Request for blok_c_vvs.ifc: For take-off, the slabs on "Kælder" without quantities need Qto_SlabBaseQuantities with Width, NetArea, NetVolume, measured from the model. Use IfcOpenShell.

First a look at what the model holds.

```python
import ifcopenshell
import ifcopenshell.util.element
import ifcopenshell.util.unit

model = ifcopenshell.open("blok_c_vvs.ifc")
print(model.schema)
for unit_type in ("LENGTHUNIT", "AREAUNIT", "VOLUMEUNIT"):
    print(unit_type, ifcopenshell.util.unit.calculate_unit_scale(model, unit_type))
storey = next(s for s in model.by_type("IfcBuildingStorey") if s.Name == "Kælder")
slabs = [e for e in ifcopenshell.util.element.get_decomposition(storey) if e.is_a("IfcSlab")]
for e in sorted(slabs, key=lambda e: e.id()):
    print(e.id(), e.is_a(), e.Name, list(ifcopenshell.util.element.get_psets(e, qtos_only=True)), sep=" | ")
```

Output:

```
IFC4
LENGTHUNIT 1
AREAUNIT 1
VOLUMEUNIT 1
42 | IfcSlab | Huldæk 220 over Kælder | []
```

```python
import ifcopenshell
import ifcopenshell.api.pset
import ifcopenshell.geom
import ifcopenshell.util.element
import ifcopenshell.util.shape
import ifcopenshell.util.unit

model = ifcopenshell.open("blok_c_vvs.ifc")
unit_scale = ifcopenshell.util.unit.calculate_unit_scale(model)
area_scale = ifcopenshell.util.unit.calculate_unit_scale(model, "AREAUNIT")
volume_scale = ifcopenshell.util.unit.calculate_unit_scale(model, "VOLUMEUNIT")
settings = ifcopenshell.geom.settings()

storey = next(s for s in model.by_type("IfcBuildingStorey") if s.Name == "Kælder")
slabs = [e for e in ifcopenshell.util.element.get_decomposition(storey) if e.is_a("IfcSlab")]

for e in sorted(slabs, key=lambda e: e.id()):
    if ifcopenshell.util.element.get_psets(e, qtos_only=True, should_inherit=False):
        continue
    # Geometry comes back in metres, in the element's own axes.
    shape = ifcopenshell.geom.create_shape(settings, e)
    values = {
        "Width": ifcopenshell.util.shape.get_z(shape.geometry) / unit_scale,
        "NetArea": ifcopenshell.util.shape.get_footprint_area(shape.geometry) / area_scale,
        "NetVolume": ifcopenshell.util.shape.get_volume(shape.geometry) / volume_scale,
    }
    qto = ifcopenshell.api.pset.add_qto(model, product=e, name="Qto_SlabBaseQuantities")
    ifcopenshell.api.pset.edit_qto(model, qto=qto, properties=values)
    print(e.id(), {k: round(v, 3) for k, v in values.items()})

model.write("blok_c_vvs_v2.ifc")
```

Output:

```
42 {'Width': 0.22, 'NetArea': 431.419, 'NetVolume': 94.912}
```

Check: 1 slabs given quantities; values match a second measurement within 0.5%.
